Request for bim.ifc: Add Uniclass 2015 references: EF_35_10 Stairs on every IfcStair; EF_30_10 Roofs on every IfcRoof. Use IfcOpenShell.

First a look at what the model holds.

```python
import ifcopenshell

model = ifcopenshell.open("bim.ifc")
print(model.schema)
print("classifications:", [c.Name for c in model.by_type("IfcClassification")])
for ifc_class in ("IfcDoor", "IfcRoof", "IfcStair", "IfcWall", "IfcWindow"):
    print(ifc_class, len(model.by_type(ifc_class)))
```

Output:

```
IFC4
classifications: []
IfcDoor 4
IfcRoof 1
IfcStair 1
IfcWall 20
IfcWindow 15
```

```python
import ifcopenshell
import ifcopenshell.api.classification

model = ifcopenshell.open("bim.ifc")

system = ifcopenshell.api.classification.add_classification(model, classification="Uniclass 2015")

codes = {
    "IfcStair": ("EF_35_10", "Stairs"),
    "IfcRoof": ("EF_30_10", "Roofs"),
}
for ifc_class, (code, name) in codes.items():
    products = model.by_type(ifc_class)
    ifcopenshell.api.classification.add_reference(
        model, products=products, classification=system, identification=code, name=name
    )
    print(code, len(products))

model.write("bim_rev.ifc")
```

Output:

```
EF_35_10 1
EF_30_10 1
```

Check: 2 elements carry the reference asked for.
